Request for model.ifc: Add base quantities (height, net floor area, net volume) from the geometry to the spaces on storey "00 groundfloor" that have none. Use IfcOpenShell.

First a look at what the model holds.

```python
import ifcopenshell
import ifcopenshell.util.element
import ifcopenshell.util.unit

model = ifcopenshell.open("model.ifc")
print(model.schema)
for unit_type in ("LENGTHUNIT", "AREAUNIT", "VOLUMEUNIT"):
    print(unit_type, ifcopenshell.util.unit.calculate_unit_scale(model, unit_type))
storey = next(s for s in model.by_type("IfcBuildingStorey") if s.Name == "00 groundfloor")
spaces = [e for e in ifcopenshell.util.element.get_decomposition(storey) if e.is_a("IfcSpace")]
for e in sorted(spaces, key=lambda e: e.id()):
    print(e.id(), e.is_a(), e.Name, list(ifcopenshell.util.element.get_psets(e, qtos_only=True)), sep=" | ")
```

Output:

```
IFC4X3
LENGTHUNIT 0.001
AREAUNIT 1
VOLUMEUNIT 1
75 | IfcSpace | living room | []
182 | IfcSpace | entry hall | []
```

```python
import ifcopenshell
import ifcopenshell.api.pset
import ifcopenshell.geom
import ifcopenshell.util.element
import ifcopenshell.util.shape
import ifcopenshell.util.unit

model = ifcopenshell.open("model.ifc")
unit_scale = ifcopenshell.util.unit.calculate_unit_scale(model)
area_scale = ifcopenshell.util.unit.calculate_unit_scale(model, "AREAUNIT")
volume_scale = ifcopenshell.util.unit.calculate_unit_scale(model, "VOLUMEUNIT")
settings = ifcopenshell.geom.settings()

storey = next(s for s in model.by_type("IfcBuildingStorey") if s.Name == "00 groundfloor")
spaces = [e for e in ifcopenshell.util.element.get_decomposition(storey) if e.is_a("IfcSpace")]

for e in sorted(spaces, key=lambda e: e.id()):
    if ifcopenshell.util.element.get_psets(e, qtos_only=True, should_inherit=False):
        continue
    # Geometry comes back in metres, in the element's own axes.
    shape = ifcopenshell.geom.create_shape(settings, e)
    values = {
        "Height": ifcopenshell.util.shape.get_z(shape.geometry) / unit_scale,
        "NetFloorArea": ifcopenshell.util.shape.get_footprint_area(shape.geometry) / area_scale,
        "NetVolume": ifcopenshell.util.shape.get_volume(shape.geometry) / volume_scale,
    }
    qto = ifcopenshell.api.pset.add_qto(model, product=e, name="Qto_SpaceBaseQuantities")
    ifcopenshell.api.pset.edit_qto(model, qto=qto, properties=values)
    print(e.id(), {k: round(v, 3) for k, v in values.items()})

model.write("model_rev.ifc")
```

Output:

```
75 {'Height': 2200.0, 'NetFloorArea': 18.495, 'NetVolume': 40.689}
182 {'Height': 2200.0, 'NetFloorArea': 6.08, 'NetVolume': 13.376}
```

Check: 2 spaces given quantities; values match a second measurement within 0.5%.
